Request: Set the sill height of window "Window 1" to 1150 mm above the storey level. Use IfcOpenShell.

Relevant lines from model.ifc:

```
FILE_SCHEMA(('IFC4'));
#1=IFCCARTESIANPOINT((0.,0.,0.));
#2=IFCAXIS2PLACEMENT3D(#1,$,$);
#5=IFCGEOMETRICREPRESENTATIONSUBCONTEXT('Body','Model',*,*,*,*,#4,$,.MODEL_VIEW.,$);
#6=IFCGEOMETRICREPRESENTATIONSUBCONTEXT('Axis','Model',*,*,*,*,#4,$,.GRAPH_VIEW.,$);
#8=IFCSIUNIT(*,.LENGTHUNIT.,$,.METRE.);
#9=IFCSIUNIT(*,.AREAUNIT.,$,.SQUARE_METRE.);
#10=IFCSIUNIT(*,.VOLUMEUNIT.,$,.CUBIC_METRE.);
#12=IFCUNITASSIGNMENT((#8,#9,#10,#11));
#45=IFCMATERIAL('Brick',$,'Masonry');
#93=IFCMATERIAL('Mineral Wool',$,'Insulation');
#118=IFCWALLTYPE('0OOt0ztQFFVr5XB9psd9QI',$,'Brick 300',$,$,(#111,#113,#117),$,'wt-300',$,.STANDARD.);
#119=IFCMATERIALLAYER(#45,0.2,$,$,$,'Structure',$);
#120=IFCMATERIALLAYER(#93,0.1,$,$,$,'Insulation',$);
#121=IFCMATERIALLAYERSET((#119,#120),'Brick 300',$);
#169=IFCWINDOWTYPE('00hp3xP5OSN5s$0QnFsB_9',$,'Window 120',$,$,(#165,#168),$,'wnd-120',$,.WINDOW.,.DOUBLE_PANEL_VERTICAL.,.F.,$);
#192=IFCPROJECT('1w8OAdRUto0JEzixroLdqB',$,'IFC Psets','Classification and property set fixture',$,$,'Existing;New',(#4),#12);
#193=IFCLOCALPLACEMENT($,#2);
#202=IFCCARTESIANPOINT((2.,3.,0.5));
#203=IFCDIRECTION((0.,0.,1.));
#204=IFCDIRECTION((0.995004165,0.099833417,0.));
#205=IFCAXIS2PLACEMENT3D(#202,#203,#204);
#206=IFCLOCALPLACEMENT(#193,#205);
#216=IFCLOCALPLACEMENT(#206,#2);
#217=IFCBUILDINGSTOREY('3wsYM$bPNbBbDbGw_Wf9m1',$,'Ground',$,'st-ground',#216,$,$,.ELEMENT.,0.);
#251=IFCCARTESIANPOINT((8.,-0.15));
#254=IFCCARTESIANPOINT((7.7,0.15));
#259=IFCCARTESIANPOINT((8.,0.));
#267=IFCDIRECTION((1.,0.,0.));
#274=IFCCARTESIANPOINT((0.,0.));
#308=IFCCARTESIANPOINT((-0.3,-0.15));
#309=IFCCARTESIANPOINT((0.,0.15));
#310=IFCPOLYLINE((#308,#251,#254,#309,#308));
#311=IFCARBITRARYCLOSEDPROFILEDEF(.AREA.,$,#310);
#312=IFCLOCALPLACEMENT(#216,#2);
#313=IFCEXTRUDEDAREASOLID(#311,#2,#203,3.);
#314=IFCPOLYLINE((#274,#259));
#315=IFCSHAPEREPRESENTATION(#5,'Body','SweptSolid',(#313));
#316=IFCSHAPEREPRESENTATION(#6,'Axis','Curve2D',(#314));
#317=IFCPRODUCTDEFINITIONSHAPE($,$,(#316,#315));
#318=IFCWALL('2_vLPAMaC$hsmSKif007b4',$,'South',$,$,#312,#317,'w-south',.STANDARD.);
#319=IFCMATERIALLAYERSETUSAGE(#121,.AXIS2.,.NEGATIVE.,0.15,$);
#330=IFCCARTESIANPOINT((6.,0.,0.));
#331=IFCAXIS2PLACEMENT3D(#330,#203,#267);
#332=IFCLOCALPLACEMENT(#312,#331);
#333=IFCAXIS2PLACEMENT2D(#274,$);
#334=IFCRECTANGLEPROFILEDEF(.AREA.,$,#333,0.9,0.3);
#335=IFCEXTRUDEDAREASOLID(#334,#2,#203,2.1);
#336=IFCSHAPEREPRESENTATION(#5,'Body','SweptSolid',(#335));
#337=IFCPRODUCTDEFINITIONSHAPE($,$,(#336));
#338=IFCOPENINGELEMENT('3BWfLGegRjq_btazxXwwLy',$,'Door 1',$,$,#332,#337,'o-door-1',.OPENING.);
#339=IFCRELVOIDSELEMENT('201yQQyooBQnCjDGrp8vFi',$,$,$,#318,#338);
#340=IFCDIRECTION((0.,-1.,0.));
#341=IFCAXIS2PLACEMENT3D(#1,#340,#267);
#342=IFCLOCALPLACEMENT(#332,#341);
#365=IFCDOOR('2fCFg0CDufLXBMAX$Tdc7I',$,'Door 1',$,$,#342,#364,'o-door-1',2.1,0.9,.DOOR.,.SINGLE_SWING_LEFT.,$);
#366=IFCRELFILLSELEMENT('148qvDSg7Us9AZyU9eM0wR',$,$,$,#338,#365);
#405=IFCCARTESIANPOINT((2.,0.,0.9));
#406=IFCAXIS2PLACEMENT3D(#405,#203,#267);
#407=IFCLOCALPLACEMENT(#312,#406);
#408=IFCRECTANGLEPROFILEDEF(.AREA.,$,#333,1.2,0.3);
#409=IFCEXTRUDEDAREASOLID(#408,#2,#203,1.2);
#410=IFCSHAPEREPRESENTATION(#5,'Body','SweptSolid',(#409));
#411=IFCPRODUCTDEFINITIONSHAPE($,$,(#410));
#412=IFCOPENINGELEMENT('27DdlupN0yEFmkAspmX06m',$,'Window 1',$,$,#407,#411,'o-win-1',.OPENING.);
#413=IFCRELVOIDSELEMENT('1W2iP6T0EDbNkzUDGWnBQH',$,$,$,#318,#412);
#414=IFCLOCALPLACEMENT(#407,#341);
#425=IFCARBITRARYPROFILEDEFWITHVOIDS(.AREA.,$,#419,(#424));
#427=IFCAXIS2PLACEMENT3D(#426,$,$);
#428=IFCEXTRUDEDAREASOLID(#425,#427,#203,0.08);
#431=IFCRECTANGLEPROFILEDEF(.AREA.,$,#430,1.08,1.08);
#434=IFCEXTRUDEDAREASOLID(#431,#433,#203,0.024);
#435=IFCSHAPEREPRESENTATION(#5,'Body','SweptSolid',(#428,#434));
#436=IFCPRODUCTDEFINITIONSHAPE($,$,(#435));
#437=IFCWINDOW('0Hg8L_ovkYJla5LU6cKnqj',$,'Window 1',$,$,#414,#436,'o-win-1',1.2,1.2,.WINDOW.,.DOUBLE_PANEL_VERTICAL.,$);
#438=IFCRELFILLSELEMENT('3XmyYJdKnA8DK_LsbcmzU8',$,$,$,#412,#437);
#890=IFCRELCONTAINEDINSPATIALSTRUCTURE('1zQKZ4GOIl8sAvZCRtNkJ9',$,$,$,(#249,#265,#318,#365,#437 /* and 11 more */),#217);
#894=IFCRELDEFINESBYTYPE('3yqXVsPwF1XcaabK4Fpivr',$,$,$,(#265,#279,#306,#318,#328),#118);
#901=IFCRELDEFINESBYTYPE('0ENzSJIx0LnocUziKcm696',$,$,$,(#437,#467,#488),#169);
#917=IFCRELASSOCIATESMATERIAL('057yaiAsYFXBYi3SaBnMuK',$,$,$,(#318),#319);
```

```python
import numpy as np
import ifcopenshell
import ifcopenshell.api.geometry
import ifcopenshell.geom
import ifcopenshell.util.element
import ifcopenshell.util.placement
import ifcopenshell.util.shape
import ifcopenshell.util.unit

model = ifcopenshell.open("model.ifc")
unit_scale = ifcopenshell.util.unit.calculate_unit_scale(model)

window = model.by_guid("0Hg8L_ovkYJla5LU6cKnqj")
opening = window.FillsVoids[0].RelatingOpeningElement
storey = ifcopenshell.util.element.get_container(window, ifc_class="IfcBuildingStorey")
level = ifcopenshell.util.placement.get_local_placement(storey.ObjectPlacement)[2, 3]

# The opening's origin need not be at the sill, so measure its lowest point.
shape = ifcopenshell.geom.create_shape(ifcopenshell.geom.settings(), opening)
bottom = ifcopenshell.util.shape.get_shape_bottom_elevation(shape, shape.geometry) / unit_scale
dz = level + 1.15 - bottom

shift = np.array([0.0, 0.0, dz])
# The window is placed relative to its opening, so it follows when the opening moves.
matrix = ifcopenshell.util.placement.get_local_placement(opening.ObjectPlacement)
matrix[:3, 3] += shift
ifcopenshell.api.geometry.edit_object_placement(
    model, product=opening, matrix=matrix, is_si=False, should_transform_children=True
)

print(f"moved by {dz * unit_scale:+.3f} m")

model.write("model_rev.ifc")
```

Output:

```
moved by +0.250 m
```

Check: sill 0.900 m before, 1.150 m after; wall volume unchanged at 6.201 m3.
